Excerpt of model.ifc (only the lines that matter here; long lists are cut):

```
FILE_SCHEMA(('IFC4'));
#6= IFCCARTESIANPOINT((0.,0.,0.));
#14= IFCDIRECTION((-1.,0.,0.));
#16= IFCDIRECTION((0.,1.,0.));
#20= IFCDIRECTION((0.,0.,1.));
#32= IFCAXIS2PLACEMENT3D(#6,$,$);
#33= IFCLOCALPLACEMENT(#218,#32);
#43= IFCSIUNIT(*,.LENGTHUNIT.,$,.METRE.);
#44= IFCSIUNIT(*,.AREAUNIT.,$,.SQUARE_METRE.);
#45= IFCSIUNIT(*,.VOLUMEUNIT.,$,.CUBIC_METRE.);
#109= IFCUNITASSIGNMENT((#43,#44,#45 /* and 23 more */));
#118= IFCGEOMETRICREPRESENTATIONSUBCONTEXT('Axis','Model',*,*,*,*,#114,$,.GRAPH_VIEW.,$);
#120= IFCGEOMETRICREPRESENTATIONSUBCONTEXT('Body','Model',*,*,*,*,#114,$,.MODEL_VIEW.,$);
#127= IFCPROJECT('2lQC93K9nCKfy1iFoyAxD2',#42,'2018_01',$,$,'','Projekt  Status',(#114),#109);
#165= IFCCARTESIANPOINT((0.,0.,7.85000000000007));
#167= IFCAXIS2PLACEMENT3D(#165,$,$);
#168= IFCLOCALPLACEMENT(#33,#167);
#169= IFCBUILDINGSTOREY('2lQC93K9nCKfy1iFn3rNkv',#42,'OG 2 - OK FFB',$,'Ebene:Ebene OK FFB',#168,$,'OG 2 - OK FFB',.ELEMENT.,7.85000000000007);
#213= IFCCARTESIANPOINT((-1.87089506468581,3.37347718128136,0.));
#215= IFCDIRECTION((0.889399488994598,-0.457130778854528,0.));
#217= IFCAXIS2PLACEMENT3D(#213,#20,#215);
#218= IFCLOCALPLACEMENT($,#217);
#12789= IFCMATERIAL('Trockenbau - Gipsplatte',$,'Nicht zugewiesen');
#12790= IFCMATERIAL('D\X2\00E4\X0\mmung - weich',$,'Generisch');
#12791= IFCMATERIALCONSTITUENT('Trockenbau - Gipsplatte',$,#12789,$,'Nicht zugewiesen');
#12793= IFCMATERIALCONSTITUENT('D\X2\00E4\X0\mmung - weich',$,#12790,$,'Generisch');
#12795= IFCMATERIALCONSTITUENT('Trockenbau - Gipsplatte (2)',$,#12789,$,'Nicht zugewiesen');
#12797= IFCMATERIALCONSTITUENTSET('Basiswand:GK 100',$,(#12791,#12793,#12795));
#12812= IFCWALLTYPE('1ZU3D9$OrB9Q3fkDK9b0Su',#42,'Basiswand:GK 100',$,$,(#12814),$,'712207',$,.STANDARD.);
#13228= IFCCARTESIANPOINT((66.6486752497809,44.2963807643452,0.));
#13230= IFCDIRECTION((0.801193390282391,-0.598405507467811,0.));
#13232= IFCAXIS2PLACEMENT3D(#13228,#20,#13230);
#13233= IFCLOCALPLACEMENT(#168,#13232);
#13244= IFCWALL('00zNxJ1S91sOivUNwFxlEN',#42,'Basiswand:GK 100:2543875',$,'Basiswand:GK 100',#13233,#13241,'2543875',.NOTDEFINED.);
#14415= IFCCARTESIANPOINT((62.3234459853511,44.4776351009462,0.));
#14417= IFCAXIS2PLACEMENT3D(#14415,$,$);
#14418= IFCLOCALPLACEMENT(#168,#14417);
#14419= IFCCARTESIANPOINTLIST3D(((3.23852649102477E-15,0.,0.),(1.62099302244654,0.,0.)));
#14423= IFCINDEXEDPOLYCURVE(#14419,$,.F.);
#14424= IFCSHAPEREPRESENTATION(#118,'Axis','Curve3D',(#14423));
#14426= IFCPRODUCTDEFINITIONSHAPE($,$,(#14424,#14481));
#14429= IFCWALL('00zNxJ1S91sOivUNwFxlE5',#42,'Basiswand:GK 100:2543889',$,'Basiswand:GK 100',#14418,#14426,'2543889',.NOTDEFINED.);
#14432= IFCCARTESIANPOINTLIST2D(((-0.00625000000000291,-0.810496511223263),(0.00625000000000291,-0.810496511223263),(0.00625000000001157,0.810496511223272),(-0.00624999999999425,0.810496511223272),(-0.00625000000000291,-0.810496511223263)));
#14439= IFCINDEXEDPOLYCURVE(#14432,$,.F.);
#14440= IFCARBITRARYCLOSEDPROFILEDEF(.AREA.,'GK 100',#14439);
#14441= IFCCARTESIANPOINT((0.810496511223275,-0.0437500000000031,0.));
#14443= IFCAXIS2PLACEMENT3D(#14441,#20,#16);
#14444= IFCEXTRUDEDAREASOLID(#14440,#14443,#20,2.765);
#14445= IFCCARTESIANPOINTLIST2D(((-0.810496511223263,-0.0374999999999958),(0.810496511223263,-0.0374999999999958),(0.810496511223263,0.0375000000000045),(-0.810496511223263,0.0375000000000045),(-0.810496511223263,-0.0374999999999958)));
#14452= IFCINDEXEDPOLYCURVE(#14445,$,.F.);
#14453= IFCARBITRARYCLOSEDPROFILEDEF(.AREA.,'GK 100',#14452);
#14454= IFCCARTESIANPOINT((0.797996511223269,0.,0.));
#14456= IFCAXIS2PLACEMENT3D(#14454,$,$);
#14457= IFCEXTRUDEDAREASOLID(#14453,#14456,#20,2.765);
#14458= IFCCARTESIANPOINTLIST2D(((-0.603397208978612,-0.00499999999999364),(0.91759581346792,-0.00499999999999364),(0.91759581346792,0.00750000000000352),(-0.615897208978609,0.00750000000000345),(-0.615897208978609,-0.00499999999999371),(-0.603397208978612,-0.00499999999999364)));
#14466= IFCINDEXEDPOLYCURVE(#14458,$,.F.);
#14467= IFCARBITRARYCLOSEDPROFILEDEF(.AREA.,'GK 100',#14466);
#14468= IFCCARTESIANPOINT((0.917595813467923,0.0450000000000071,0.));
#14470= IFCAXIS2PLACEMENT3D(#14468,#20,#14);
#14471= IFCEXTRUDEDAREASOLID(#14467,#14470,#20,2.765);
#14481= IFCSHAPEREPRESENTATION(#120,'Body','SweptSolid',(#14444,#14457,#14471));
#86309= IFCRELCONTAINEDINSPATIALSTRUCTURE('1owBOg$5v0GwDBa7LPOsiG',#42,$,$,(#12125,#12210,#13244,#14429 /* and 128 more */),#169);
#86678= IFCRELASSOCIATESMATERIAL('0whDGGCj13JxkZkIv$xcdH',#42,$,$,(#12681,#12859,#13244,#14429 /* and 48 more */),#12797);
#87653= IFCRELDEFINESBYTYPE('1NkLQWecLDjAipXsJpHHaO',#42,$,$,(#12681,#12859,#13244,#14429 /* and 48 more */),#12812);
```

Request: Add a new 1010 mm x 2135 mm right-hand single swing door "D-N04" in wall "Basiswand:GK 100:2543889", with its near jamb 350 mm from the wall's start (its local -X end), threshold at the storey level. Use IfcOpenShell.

```python
import numpy as np
import ifcopenshell
import ifcopenshell.api.feature
import ifcopenshell.api.geometry
import ifcopenshell.api.root
import ifcopenshell.api.spatial
import ifcopenshell.geom
import ifcopenshell.util.element
import ifcopenshell.util.placement
import ifcopenshell.util.representation
import ifcopenshell.util.shape
import ifcopenshell.util.unit

model = ifcopenshell.open("model.ifc")
unit_scale = ifcopenshell.util.unit.calculate_unit_scale(model)
settings = ifcopenshell.geom.settings()


def volume(element):
    """Net volume in cubic metres, openings subtracted."""
    shape = ifcopenshell.geom.create_shape(settings, element)
    return ifcopenshell.util.shape.get_volume(shape.geometry)


wall = model.by_id(14429)
storey = ifcopenshell.util.element.get_container(wall, ifc_class="IfcBuildingStorey")
context = ifcopenshell.util.representation.get_context(model, "Model", "Body", "MODEL_VIEW")
before = volume(wall)

width, height, from_end, sill = 1.01, 2.135, 0.35, 0.0  # metres

# The wall runs along its own X axis, and the end named is its -X end.
wall_shape = ifcopenshell.geom.create_shape(settings, wall)
x, y, z = ifcopenshell.util.shape.get_vertices(wall_shape.geometry).T
start = x.min() + from_end
face, thickness = float(y.min()), float(y.max() - y.min())
wall_matrix = ifcopenshell.util.placement.get_local_placement(wall.ObjectPlacement)
level = ifcopenshell.util.placement.get_local_placement(storey.ObjectPlacement)[2, 3]


def in_wall(x, y):
    """Placement at x, y metres in the wall's axes, at sill height."""
    matrix = wall_matrix.copy()
    matrix[:, 3] = wall_matrix @ np.array([x / unit_scale, y / unit_scale, 0.0, 1.0])
    matrix[2, 3] = level + sill / unit_scale
    return matrix


# Opening: a box that overshoots both wall faces by 50 mm.
opening = ifcopenshell.api.root.create_entity(model, ifc_class="IfcOpeningElement", predefined_type="OPENING")
box = ifcopenshell.api.geometry.add_wall_representation(
    model, context=context, length=width, height=height, thickness=thickness + 0.1
)
ifcopenshell.api.geometry.assign_representation(model, product=opening, representation=box)
ifcopenshell.api.geometry.edit_object_placement(model, product=opening, matrix=in_wall(start, face - 0.05), is_si=False)
ifcopenshell.api.feature.add_feature(model, feature=opening, element=wall)

door = ifcopenshell.api.root.create_entity(model, ifc_class="IfcDoor", name="D-N04", predefined_type="DOOR")
door.OverallWidth, door.OverallHeight = width / unit_scale, height / unit_scale
door.OperationType = "SINGLE_SWING_RIGHT"
body = ifcopenshell.api.geometry.add_door_representation(
    model,
    context=context,
    overall_width=door.OverallWidth,
    overall_height=door.OverallHeight,
    operation_type="SINGLE_SWING_RIGHT",
    lining_properties={"LiningDepth": thickness / unit_scale, "ThresholdDepth": thickness / unit_scale},
)
ifcopenshell.api.geometry.assign_representation(model, product=door, representation=body)
ifcopenshell.api.spatial.assign_container(model, products=[door], relating_structure=storey)
ifcopenshell.api.feature.add_filling(model, opening=opening, element=door)

# The lining spans the wall, so the door starts at the wall face.
ifcopenshell.api.geometry.edit_object_placement(model, product=door, matrix=in_wall(start, face), is_si=False)

after = volume(wall)

print(f"wall volume {before:.3f} -> {after:.3f} m3")

model.write("model_rev.ifc")
```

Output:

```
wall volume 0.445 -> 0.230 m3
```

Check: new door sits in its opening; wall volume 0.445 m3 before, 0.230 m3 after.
